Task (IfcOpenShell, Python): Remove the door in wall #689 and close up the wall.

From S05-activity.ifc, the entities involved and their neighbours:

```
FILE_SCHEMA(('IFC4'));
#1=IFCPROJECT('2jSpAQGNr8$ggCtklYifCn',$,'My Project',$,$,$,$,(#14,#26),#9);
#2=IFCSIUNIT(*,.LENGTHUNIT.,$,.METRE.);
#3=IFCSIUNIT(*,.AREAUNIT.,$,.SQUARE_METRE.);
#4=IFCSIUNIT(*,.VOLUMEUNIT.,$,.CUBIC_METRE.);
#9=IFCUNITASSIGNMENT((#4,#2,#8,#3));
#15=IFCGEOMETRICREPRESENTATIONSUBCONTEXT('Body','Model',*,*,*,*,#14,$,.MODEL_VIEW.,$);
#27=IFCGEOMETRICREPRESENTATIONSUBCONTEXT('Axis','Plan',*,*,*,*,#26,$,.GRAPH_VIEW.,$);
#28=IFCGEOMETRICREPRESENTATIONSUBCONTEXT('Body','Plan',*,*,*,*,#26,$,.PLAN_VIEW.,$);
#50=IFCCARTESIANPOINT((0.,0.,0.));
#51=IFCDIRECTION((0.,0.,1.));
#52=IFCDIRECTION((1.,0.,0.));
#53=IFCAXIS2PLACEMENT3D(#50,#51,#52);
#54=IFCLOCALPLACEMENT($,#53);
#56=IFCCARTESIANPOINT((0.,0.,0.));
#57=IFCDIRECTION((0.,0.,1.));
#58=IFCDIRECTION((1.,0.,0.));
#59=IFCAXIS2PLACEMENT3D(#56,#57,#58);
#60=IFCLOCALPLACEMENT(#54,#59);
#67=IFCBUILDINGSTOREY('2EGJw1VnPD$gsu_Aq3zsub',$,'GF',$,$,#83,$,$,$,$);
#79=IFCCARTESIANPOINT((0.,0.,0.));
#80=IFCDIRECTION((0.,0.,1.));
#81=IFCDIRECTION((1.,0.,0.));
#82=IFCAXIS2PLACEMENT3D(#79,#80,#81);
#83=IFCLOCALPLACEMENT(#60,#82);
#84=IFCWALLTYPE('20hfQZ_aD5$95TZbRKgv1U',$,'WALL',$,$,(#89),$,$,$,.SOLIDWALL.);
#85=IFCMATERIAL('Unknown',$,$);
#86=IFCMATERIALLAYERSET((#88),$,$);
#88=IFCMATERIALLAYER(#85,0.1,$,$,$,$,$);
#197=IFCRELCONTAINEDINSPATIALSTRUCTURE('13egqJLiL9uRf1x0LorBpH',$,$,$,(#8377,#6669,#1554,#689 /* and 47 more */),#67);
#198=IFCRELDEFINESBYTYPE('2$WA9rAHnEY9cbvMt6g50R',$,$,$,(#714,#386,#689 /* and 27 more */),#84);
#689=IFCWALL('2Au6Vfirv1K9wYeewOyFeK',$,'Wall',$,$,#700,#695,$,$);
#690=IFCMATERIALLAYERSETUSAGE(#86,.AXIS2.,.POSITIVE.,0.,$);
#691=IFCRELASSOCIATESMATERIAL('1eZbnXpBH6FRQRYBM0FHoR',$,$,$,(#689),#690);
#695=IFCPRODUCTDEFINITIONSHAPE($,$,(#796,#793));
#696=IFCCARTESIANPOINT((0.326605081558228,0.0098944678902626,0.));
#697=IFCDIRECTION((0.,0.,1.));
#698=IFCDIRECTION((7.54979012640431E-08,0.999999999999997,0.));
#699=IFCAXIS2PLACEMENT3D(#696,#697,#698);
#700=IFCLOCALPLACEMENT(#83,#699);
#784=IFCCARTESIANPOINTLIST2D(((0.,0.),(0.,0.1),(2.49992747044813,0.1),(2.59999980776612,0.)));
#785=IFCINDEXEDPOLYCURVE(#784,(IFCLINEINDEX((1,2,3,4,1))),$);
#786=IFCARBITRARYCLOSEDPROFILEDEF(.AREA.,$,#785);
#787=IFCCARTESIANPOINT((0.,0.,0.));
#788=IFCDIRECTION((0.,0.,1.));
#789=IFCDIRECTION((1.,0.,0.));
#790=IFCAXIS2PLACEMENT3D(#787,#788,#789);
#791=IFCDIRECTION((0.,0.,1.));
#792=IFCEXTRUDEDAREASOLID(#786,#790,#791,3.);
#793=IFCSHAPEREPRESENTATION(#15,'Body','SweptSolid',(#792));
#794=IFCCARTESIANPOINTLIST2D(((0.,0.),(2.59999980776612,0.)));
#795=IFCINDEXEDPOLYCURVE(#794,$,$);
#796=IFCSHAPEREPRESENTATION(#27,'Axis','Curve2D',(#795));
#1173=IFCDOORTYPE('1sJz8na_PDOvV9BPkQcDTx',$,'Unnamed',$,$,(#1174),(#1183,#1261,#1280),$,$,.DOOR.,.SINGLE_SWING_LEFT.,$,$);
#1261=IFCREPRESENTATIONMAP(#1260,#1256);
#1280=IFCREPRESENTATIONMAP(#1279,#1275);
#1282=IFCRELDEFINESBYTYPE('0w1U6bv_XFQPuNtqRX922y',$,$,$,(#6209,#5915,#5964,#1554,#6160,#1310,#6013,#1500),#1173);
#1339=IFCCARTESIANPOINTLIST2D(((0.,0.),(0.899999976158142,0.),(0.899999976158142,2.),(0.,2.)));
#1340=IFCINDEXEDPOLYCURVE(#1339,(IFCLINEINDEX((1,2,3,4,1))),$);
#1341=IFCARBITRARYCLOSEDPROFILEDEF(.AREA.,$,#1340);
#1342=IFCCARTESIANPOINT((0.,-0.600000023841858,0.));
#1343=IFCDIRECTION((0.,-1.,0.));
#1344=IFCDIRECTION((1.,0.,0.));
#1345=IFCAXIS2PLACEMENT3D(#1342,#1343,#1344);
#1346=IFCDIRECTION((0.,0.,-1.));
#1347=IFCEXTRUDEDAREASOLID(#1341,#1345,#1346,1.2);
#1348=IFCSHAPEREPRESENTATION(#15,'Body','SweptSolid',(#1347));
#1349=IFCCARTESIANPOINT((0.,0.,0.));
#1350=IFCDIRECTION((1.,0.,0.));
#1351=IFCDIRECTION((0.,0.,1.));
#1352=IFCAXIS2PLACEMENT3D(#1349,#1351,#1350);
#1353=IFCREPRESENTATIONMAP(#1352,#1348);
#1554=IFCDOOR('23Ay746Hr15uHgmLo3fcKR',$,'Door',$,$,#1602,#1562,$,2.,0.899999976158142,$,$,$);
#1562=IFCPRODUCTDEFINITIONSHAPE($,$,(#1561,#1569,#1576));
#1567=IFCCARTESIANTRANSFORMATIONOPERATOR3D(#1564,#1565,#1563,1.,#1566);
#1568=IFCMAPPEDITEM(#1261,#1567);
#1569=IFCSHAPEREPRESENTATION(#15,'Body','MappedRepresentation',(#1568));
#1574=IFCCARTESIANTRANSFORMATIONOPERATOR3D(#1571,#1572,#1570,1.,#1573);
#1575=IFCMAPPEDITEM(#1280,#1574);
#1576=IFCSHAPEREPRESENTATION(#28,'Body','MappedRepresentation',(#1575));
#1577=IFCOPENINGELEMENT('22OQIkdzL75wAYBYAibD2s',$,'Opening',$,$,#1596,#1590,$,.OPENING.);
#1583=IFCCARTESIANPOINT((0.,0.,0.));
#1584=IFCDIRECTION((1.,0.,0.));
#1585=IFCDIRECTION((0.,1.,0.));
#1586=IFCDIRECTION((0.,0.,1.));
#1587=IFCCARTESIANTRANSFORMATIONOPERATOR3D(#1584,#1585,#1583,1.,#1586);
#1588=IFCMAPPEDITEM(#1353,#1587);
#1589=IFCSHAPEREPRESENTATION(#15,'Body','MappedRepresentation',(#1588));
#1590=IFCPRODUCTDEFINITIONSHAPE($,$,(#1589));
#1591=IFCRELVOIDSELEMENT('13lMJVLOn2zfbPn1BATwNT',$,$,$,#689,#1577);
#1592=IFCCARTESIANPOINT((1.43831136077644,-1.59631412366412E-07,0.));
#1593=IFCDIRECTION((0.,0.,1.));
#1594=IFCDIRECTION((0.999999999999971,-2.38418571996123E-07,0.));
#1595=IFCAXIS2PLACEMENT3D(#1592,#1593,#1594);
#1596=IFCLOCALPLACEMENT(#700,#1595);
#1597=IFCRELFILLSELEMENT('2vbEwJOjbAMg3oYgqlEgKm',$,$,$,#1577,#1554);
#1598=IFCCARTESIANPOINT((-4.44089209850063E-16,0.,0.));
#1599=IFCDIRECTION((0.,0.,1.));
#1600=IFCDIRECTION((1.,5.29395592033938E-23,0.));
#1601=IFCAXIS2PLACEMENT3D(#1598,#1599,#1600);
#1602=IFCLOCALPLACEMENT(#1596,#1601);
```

```python
import ifcopenshell
import ifcopenshell.api.feature
import ifcopenshell.api.root
import ifcopenshell.geom
import ifcopenshell.util.shape

model = ifcopenshell.open("S05-activity.ifc")
settings = ifcopenshell.geom.settings()


def volume(element):
    """Net volume in cubic metres, openings subtracted."""
    shape = ifcopenshell.geom.create_shape(settings, element)
    return ifcopenshell.util.shape.get_volume(shape.geometry)


door = model.by_guid("23Ay746Hr15uHgmLo3fcKR")
opening = door.FillsVoids[0].RelatingOpeningElement
wall = opening.VoidsElements[0].RelatingBuildingElement
before = volume(wall)

ifcopenshell.api.root.remove_product(model, product=door)
ifcopenshell.api.feature.remove_feature(model, feature=opening)

after = volume(wall)

print(f"wall volume {before:.3f} -> {after:.3f} m3")

model.write("S05-activity_v2.ifc")
```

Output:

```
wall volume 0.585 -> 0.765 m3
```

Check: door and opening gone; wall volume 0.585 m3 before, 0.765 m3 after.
